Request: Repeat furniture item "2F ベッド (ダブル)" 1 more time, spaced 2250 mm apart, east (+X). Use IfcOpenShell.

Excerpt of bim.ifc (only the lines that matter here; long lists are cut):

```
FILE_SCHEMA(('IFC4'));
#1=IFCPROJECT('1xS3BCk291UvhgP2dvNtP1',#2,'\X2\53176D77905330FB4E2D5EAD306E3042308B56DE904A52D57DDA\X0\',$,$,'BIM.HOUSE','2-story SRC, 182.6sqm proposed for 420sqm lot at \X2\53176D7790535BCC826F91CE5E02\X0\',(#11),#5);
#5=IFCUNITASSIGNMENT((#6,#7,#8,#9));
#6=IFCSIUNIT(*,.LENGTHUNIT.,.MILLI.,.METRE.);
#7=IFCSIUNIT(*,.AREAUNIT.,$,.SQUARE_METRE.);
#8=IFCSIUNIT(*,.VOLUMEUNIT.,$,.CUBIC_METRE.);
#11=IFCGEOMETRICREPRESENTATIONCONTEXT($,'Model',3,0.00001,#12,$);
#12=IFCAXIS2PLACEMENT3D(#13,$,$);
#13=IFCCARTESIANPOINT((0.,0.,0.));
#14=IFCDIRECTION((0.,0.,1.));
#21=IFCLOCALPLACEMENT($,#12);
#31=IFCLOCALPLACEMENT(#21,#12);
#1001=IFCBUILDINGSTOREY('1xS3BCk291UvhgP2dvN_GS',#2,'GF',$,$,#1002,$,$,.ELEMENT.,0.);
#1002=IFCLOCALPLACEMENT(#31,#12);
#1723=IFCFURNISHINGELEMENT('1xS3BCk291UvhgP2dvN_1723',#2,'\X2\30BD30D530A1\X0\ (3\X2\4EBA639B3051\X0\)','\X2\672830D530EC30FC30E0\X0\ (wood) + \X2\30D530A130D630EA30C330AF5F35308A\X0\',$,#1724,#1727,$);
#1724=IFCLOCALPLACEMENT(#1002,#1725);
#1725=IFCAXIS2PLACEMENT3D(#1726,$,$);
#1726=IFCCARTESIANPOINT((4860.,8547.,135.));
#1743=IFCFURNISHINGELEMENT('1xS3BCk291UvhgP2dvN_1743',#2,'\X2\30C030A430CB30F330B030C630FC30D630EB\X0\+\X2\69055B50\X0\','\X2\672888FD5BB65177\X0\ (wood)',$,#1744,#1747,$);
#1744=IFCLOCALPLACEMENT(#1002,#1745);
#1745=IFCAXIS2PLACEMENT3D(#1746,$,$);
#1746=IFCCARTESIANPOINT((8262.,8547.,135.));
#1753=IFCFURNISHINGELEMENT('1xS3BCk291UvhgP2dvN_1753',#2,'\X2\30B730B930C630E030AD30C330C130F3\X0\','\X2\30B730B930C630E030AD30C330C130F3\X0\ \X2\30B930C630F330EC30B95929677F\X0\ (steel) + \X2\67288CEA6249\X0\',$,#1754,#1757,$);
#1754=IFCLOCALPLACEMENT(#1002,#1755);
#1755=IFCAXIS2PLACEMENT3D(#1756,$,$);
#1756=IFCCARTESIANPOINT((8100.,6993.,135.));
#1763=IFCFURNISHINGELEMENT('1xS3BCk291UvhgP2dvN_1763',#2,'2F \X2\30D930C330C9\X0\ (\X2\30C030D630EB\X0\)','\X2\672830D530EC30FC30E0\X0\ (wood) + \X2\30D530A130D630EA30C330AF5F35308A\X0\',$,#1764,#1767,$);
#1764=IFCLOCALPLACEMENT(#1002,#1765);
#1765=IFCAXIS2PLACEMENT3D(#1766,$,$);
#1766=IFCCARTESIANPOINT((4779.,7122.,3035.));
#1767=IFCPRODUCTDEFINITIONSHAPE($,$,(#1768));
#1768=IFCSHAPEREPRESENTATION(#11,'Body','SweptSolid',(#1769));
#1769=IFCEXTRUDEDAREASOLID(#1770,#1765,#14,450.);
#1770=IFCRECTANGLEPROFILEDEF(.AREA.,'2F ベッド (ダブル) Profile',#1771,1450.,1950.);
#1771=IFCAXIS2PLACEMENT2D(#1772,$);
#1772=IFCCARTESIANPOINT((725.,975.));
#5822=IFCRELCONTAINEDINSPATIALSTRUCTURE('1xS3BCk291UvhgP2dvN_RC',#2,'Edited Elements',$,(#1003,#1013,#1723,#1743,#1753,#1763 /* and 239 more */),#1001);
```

```python
import numpy as np
import ifcopenshell
import ifcopenshell.api.geometry
import ifcopenshell.api.root
import ifcopenshell.util.element
import ifcopenshell.util.placement
import ifcopenshell.util.unit

model = ifcopenshell.open("bim.ifc")
unit_scale = ifcopenshell.util.unit.calculate_unit_scale(model)


def reuse_history(source, copy):
    """copy_class also copies each property set's owner history, people and application; keep the originals."""
    for rel in copy.IsDefinedBy:
        if rel.is_a("IfcRelDefinesByProperties") and (history := rel.RelatingPropertyDefinition.OwnerHistory):
            rel.RelatingPropertyDefinition.OwnerHistory = source.OwnerHistory
            ifcopenshell.util.element.remove_deep2(model, history)


source = model.by_guid("1xS3BCk291UvhgP2dvN_1763")
base = ifcopenshell.util.placement.get_local_placement(source.ObjectPlacement)
step = np.array([1.0, 0.0, 0.0]) * 2.25 / unit_scale

for i in range(1, 2):
    copy = ifcopenshell.api.root.copy_class(model, product=source)
    copy.Representation = ifcopenshell.util.element.copy_deep(
        model, source.Representation, exclude=["IfcGeometricRepresentationContext", "IfcRepresentationMap"]
    )
    reuse_history(source, copy)
    matrix = base.copy()
    matrix[:3, 3] += i * step
    print("added at", matrix[:3, 3].round(3) + 0.0)
    ifcopenshell.api.geometry.edit_object_placement(model, product=copy, matrix=matrix, is_si=False)

model.write("bim_edited.ifc")
```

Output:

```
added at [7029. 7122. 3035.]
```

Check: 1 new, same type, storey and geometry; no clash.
